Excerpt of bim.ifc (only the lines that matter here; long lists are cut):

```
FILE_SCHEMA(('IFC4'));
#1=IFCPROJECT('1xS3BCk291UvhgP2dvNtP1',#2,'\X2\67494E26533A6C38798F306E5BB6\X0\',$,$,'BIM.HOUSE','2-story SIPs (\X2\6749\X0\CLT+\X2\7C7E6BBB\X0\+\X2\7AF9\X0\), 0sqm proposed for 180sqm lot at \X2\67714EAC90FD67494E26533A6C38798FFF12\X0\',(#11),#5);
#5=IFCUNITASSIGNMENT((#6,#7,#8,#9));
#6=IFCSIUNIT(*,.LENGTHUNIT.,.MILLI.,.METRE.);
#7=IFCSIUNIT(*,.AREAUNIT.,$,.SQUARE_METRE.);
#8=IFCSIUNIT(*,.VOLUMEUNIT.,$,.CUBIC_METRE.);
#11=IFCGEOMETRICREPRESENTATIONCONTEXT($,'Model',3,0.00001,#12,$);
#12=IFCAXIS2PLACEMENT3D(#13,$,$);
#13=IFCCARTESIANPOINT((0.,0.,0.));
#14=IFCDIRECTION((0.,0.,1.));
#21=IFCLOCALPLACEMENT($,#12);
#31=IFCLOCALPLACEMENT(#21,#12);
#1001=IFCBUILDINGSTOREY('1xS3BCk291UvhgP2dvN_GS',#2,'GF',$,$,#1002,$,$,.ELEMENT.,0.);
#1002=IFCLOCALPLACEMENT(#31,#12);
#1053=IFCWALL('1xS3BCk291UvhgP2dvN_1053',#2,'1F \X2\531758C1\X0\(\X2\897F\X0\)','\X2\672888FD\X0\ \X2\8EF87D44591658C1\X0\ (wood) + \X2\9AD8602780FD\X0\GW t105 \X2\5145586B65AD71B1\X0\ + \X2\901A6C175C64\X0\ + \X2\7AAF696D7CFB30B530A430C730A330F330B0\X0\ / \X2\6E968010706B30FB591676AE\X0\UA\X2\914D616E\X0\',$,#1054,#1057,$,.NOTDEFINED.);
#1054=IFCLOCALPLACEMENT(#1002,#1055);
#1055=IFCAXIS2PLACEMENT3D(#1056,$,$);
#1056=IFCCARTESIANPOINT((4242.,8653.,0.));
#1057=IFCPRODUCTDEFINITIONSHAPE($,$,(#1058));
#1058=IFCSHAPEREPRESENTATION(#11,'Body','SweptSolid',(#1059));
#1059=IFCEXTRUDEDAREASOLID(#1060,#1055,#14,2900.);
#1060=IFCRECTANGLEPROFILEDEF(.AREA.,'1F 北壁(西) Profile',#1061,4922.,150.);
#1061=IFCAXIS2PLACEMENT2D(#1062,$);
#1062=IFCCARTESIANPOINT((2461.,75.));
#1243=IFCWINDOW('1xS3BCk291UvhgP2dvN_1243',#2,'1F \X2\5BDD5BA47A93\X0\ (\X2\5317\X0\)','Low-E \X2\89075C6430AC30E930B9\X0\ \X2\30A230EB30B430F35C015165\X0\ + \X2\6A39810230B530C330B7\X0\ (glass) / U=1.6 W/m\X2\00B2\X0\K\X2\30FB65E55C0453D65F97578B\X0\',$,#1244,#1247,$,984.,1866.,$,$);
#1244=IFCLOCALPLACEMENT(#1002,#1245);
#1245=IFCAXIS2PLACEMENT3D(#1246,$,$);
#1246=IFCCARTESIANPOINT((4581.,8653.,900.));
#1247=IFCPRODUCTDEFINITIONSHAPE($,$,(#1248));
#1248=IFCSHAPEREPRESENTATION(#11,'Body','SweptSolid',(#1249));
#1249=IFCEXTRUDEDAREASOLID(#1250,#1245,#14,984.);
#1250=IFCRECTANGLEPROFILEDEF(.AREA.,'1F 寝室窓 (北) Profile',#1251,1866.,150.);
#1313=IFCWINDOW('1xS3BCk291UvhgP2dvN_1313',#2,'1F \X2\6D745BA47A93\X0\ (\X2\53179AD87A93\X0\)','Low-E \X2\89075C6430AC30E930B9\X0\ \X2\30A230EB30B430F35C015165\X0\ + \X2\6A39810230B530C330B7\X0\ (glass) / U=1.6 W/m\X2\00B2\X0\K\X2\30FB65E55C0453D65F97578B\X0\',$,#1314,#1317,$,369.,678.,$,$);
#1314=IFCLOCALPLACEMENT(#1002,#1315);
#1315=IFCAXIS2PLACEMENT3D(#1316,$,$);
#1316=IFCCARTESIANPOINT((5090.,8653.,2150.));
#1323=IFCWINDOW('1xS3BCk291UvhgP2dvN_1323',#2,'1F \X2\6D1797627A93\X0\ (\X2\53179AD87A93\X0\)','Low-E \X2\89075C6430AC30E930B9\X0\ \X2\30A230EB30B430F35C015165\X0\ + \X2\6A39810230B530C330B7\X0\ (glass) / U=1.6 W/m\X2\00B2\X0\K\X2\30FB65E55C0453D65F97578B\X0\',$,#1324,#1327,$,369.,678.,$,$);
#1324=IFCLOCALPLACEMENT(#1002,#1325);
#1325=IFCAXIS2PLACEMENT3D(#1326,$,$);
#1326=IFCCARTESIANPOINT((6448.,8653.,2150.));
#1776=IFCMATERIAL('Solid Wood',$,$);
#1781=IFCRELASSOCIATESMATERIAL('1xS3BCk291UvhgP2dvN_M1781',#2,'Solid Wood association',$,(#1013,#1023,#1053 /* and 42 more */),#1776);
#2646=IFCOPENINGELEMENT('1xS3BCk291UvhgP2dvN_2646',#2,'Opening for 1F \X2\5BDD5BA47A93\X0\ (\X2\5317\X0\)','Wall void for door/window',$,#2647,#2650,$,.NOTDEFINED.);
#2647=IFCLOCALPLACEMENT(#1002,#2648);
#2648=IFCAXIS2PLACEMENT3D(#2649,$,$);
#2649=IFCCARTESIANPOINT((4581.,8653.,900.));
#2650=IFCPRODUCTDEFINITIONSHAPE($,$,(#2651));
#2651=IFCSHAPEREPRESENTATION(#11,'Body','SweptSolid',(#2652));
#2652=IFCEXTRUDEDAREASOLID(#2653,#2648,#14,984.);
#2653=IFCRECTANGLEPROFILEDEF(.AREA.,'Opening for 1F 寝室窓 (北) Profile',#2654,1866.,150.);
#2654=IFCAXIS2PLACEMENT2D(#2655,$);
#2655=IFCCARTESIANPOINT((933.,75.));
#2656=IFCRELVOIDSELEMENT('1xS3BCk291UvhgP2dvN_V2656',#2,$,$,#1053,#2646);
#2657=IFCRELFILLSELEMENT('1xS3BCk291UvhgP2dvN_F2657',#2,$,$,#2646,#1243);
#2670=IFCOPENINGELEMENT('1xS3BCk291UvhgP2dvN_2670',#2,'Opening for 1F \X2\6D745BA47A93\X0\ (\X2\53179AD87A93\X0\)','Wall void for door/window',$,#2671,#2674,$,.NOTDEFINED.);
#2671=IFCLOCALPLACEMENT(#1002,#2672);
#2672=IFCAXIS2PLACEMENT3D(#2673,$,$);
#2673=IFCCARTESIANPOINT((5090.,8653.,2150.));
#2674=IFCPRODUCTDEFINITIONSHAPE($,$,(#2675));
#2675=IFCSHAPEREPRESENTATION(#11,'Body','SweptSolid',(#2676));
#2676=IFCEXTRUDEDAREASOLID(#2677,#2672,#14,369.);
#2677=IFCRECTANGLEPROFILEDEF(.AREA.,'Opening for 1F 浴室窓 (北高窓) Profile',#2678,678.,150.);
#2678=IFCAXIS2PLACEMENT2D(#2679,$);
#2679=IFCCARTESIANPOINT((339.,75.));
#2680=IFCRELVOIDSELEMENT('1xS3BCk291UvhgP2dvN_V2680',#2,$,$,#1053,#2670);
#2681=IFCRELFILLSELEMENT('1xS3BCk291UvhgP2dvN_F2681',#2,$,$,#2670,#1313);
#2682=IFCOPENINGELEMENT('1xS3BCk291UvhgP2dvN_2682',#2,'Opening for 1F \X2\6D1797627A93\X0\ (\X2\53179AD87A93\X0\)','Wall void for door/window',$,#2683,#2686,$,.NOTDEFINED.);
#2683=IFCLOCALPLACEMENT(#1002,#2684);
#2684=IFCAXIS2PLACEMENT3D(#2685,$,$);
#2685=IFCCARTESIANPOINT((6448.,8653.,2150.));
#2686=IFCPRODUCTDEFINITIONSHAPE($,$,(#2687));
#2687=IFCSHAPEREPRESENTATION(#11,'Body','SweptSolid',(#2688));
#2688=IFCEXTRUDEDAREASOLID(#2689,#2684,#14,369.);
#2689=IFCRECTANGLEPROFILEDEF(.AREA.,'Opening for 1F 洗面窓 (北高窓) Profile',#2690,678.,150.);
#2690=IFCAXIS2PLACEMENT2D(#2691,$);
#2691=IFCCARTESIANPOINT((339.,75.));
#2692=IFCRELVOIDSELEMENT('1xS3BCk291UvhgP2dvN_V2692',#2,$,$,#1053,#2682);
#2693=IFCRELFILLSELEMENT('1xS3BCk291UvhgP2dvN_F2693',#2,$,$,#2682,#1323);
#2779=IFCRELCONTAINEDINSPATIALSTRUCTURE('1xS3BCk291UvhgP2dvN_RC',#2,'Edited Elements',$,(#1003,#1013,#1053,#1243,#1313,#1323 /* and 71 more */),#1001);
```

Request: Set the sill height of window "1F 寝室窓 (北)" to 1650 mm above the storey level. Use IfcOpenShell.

```python
import numpy as np
import ifcopenshell
import ifcopenshell.api.geometry
import ifcopenshell.geom
import ifcopenshell.util.element
import ifcopenshell.util.placement
import ifcopenshell.util.shape
import ifcopenshell.util.unit

model = ifcopenshell.open("bim.ifc")
unit_scale = ifcopenshell.util.unit.calculate_unit_scale(model)

window = model.by_guid("1xS3BCk291UvhgP2dvN_1243")
opening = window.FillsVoids[0].RelatingOpeningElement
storey = ifcopenshell.util.element.get_container(window, ifc_class="IfcBuildingStorey")
level = ifcopenshell.util.placement.get_local_placement(storey.ObjectPlacement)[2, 3]

# The opening's origin need not be at the sill, so measure its lowest point.
shape = ifcopenshell.geom.create_shape(ifcopenshell.geom.settings(), opening)
bottom = ifcopenshell.util.shape.get_shape_bottom_elevation(shape, shape.geometry) / unit_scale
dz = level + 1.65 / unit_scale - bottom

shift = np.array([0.0, 0.0, dz])
# The window is not placed relative to its opening, so move both.
for product in (opening, window):
    matrix = ifcopenshell.util.placement.get_local_placement(product.ObjectPlacement)
    matrix[:3, 3] += shift
    ifcopenshell.api.geometry.edit_object_placement(model, product=product, matrix=matrix, is_si=False)

print(f"moved by {dz * unit_scale:+.3f} m")

model.write("bim_rev.ifc")
```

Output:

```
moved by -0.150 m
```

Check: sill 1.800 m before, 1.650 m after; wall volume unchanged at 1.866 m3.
